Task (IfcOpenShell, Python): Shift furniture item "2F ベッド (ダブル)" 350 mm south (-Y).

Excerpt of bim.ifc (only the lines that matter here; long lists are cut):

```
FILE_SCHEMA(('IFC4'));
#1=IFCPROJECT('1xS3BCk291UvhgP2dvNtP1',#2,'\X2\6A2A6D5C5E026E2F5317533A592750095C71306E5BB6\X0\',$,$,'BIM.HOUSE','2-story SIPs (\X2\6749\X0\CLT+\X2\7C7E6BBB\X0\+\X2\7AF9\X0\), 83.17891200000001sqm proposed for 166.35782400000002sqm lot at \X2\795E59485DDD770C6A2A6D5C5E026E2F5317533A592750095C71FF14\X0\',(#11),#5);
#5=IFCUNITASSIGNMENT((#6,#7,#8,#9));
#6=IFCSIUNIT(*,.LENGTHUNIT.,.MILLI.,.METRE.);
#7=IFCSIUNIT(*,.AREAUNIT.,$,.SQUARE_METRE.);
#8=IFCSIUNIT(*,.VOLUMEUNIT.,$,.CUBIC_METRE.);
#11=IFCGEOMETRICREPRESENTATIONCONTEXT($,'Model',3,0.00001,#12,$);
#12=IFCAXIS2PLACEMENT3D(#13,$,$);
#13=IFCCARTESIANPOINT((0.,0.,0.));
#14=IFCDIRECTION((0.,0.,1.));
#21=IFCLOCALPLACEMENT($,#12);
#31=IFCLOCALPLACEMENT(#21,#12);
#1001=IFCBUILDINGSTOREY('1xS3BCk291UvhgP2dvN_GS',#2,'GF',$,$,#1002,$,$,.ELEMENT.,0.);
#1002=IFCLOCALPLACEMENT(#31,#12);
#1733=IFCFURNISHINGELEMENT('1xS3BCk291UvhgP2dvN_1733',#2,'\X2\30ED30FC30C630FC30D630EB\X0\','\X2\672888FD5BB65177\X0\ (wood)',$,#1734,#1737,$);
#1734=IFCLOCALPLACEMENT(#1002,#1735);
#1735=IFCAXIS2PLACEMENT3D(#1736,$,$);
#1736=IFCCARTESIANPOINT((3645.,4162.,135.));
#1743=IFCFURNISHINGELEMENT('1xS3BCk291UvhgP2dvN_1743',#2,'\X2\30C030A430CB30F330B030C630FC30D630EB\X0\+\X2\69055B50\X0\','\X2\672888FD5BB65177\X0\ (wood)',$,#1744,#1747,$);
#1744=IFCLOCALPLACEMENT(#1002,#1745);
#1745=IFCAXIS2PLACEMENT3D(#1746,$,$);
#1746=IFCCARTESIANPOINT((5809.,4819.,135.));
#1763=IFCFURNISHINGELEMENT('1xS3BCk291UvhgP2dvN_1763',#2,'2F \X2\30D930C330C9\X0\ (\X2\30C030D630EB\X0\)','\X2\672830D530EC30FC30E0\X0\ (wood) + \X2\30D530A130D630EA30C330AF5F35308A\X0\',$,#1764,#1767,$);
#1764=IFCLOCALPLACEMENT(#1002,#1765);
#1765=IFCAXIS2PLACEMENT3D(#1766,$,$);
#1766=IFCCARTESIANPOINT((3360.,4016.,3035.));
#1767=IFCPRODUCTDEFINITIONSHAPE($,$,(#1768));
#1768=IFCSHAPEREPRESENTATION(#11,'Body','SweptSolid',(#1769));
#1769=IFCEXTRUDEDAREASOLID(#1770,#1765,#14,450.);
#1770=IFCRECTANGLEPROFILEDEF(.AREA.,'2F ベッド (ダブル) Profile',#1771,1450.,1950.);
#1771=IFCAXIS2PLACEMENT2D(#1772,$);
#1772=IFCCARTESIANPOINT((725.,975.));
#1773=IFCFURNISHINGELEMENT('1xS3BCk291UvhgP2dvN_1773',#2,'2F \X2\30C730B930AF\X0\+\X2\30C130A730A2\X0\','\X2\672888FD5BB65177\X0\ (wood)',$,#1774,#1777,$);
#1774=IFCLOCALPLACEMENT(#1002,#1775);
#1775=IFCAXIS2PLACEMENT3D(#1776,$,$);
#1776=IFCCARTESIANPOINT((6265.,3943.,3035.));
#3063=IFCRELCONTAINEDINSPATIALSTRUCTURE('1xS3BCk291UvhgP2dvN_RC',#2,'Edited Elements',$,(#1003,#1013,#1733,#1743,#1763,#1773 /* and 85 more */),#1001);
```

```python
import ifcopenshell
import ifcopenshell.api.geometry
import ifcopenshell.util.placement
import ifcopenshell.util.unit

model = ifcopenshell.open("bim.ifc")
unit_scale = ifcopenshell.util.unit.calculate_unit_scale(model)

item = model.by_guid("1xS3BCk291UvhgP2dvN_1763")
matrix = ifcopenshell.util.placement.get_local_placement(item.ObjectPlacement)
matrix[1, 3] -= 0.35 / unit_scale
ifcopenshell.api.geometry.edit_object_placement(model, product=item, matrix=matrix, is_si=False)

print(ifcopenshell.util.placement.get_local_placement(item.ObjectPlacement).round(3) + 0.0)

model.write("bim_updated.ifc")
```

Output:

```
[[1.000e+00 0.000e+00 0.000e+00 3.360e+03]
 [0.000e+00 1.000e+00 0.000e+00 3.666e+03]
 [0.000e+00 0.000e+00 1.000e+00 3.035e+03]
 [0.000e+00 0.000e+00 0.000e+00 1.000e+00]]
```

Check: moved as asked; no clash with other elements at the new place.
